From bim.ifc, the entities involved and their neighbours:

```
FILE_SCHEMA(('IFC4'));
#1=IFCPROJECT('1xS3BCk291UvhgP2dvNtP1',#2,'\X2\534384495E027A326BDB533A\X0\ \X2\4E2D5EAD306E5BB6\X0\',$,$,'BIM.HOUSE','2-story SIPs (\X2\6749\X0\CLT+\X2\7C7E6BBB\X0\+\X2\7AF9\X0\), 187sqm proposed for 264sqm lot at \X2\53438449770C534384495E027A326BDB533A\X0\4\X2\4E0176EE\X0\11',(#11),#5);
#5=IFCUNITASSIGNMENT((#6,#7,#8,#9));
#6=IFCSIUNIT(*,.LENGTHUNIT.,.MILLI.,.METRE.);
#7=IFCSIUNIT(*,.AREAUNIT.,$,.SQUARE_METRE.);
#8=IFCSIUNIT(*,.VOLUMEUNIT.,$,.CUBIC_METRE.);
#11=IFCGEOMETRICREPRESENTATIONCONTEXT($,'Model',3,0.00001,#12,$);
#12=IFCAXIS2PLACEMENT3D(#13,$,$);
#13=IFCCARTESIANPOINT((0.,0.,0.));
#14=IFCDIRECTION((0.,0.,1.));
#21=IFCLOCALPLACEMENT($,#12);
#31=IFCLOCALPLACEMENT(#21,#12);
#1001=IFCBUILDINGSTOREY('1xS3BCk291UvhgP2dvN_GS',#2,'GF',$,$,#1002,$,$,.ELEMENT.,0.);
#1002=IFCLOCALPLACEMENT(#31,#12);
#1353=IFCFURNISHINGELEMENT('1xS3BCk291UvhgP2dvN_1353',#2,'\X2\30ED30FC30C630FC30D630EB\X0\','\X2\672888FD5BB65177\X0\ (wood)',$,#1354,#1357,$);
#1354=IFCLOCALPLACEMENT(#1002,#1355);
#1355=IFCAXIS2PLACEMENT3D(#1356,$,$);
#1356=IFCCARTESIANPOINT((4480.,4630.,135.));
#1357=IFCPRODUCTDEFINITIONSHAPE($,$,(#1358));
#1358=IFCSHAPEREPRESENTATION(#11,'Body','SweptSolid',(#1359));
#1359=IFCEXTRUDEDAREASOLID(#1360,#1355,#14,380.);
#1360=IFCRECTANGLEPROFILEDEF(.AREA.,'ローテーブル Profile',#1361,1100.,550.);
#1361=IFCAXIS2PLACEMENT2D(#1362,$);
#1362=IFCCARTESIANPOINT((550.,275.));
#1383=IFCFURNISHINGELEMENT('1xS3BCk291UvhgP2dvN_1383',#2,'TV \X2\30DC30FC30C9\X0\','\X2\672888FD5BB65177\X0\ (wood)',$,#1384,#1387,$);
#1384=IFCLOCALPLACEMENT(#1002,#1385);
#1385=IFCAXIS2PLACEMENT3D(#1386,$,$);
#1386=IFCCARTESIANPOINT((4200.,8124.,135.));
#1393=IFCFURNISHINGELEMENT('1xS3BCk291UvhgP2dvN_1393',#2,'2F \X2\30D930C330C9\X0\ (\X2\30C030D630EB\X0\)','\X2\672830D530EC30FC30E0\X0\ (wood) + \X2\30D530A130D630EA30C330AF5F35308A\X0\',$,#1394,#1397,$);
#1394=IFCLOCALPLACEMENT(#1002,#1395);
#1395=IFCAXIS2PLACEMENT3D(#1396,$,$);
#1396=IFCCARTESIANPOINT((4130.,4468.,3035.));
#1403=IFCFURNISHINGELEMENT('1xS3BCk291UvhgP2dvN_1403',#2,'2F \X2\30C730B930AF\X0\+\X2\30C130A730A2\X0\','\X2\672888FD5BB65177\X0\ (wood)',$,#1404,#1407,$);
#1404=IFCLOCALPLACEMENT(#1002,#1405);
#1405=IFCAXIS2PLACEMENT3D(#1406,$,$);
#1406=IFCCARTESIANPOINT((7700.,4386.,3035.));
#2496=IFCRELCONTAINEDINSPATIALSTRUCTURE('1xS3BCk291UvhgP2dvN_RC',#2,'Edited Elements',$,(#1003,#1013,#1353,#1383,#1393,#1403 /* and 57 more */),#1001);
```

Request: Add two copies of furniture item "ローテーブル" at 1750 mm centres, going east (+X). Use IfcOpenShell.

```python
import numpy as np
import ifcopenshell
import ifcopenshell.api.geometry
import ifcopenshell.api.root
import ifcopenshell.util.element
import ifcopenshell.util.placement
import ifcopenshell.util.unit

model = ifcopenshell.open("bim.ifc")
unit_scale = ifcopenshell.util.unit.calculate_unit_scale(model)


def reuse_history(source, copy):
    """copy_class also copies each property set's owner history, people and application; keep the originals."""
    for rel in copy.IsDefinedBy:
        if rel.is_a("IfcRelDefinesByProperties") and (history := rel.RelatingPropertyDefinition.OwnerHistory):
            rel.RelatingPropertyDefinition.OwnerHistory = source.OwnerHistory
            ifcopenshell.util.element.remove_deep2(model, history)


source = model.by_guid("1xS3BCk291UvhgP2dvN_1353")
base = ifcopenshell.util.placement.get_local_placement(source.ObjectPlacement)
step = np.array([1.0, 0.0, 0.0]) * 1.75 / unit_scale

for i in range(1, 3):
    copy = ifcopenshell.api.root.copy_class(model, product=source)
    copy.Representation = ifcopenshell.util.element.copy_deep(
        model, source.Representation, exclude=["IfcGeometricRepresentationContext", "IfcRepresentationMap"]
    )
    reuse_history(source, copy)
    matrix = base.copy()
    matrix[:3, 3] += i * step
    print("added at", matrix[:3, 3].round(3) + 0.0)
    ifcopenshell.api.geometry.edit_object_placement(model, product=copy, matrix=matrix, is_si=False)

model.write("bim_edited.ifc")
```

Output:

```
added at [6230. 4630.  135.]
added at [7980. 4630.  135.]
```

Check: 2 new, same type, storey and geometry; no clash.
